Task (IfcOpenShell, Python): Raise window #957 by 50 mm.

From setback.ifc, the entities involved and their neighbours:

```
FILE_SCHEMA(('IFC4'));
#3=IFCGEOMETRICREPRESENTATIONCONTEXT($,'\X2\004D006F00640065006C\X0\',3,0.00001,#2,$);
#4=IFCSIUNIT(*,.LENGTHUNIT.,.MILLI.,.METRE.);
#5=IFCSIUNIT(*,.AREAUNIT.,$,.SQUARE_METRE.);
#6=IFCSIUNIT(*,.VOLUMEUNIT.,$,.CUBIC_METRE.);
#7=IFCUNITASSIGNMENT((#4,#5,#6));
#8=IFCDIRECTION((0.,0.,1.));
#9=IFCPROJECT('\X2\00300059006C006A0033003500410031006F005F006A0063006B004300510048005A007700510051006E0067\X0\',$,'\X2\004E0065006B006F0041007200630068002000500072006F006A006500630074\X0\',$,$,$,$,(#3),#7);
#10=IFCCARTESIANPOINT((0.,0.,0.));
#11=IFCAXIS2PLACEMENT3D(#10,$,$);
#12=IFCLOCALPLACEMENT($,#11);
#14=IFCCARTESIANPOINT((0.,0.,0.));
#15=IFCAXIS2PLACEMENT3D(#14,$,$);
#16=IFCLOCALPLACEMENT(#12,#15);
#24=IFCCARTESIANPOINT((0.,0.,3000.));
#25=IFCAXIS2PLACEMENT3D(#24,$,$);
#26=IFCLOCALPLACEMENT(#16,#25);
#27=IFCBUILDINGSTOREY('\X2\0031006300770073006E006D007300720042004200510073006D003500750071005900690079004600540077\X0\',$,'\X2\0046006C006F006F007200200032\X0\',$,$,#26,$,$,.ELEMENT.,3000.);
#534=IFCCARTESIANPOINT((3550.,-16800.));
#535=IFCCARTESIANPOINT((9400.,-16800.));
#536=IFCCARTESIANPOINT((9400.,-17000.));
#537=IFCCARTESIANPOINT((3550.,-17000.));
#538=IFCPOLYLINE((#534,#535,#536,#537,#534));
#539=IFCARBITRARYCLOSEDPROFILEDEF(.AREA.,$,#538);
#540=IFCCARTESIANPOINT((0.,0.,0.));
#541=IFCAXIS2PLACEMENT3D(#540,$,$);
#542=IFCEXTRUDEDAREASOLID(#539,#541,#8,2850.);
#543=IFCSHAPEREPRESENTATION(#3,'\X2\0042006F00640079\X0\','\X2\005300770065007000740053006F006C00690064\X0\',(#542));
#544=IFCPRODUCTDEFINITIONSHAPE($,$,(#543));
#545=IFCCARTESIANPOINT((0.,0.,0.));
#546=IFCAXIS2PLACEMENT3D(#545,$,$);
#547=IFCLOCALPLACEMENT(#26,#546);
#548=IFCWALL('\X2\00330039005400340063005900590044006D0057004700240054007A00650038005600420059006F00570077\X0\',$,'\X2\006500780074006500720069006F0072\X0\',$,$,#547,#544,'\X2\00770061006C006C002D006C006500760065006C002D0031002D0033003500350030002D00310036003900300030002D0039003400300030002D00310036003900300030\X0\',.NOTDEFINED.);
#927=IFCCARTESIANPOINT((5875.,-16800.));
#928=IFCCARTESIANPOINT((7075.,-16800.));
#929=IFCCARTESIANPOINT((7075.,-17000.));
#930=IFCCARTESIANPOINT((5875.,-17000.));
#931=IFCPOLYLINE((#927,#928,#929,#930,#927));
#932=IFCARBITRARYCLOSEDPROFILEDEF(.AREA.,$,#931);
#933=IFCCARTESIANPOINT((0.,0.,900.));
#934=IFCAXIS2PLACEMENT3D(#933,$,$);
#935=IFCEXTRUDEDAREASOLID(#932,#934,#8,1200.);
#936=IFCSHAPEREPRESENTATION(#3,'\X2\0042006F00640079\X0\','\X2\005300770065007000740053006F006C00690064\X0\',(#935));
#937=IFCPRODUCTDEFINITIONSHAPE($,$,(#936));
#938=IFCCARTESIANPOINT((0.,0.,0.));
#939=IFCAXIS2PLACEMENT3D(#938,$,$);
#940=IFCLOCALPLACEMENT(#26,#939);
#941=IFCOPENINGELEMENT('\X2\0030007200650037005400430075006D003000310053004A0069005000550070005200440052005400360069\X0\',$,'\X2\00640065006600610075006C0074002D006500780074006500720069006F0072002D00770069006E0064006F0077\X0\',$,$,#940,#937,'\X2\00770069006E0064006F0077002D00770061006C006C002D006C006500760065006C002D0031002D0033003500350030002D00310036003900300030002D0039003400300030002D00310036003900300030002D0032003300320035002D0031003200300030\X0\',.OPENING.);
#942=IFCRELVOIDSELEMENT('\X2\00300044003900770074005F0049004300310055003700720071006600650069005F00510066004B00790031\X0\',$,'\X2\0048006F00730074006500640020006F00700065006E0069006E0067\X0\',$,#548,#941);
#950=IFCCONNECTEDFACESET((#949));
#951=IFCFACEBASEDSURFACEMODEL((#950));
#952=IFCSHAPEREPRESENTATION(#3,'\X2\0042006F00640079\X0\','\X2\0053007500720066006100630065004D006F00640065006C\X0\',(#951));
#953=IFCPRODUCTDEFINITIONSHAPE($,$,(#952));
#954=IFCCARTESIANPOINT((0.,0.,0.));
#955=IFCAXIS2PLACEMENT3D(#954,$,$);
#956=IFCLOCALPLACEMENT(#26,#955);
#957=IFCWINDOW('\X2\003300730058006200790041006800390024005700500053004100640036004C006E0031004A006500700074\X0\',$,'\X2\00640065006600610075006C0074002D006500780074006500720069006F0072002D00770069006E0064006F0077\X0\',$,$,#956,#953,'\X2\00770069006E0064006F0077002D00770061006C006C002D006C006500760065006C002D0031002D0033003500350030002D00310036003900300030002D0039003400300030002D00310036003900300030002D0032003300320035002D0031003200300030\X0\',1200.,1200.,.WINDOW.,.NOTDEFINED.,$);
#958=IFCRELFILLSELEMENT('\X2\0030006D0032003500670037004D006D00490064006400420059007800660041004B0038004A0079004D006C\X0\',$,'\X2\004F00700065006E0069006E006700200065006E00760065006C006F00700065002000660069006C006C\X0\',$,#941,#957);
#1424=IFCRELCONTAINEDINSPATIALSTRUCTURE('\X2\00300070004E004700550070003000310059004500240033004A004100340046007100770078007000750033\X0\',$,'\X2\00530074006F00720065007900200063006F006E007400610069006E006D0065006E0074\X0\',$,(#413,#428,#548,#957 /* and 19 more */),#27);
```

```python
import numpy as np
import ifcopenshell
import ifcopenshell.api.geometry
import ifcopenshell.util.placement
import ifcopenshell.util.unit

model = ifcopenshell.open("setback.ifc")
unit_scale = ifcopenshell.util.unit.calculate_unit_scale(model)

window = model.by_guid("3sXbyAh9$WPSAd6Ln1Jept")
opening = window.FillsVoids[0].RelatingOpeningElement
dz = 0.05 / unit_scale

shift = np.array([0.0, 0.0, dz])
# The window is not placed relative to its opening, so move both.
for product in (opening, window):
    matrix = ifcopenshell.util.placement.get_local_placement(product.ObjectPlacement)
    matrix[:3, 3] += shift
    ifcopenshell.api.geometry.edit_object_placement(model, product=product, matrix=matrix, is_si=False)

print(f"moved by {dz * unit_scale:+.3f} m")

model.write("setback-out.ifc")
```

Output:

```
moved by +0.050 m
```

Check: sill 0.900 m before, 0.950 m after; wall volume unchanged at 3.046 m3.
